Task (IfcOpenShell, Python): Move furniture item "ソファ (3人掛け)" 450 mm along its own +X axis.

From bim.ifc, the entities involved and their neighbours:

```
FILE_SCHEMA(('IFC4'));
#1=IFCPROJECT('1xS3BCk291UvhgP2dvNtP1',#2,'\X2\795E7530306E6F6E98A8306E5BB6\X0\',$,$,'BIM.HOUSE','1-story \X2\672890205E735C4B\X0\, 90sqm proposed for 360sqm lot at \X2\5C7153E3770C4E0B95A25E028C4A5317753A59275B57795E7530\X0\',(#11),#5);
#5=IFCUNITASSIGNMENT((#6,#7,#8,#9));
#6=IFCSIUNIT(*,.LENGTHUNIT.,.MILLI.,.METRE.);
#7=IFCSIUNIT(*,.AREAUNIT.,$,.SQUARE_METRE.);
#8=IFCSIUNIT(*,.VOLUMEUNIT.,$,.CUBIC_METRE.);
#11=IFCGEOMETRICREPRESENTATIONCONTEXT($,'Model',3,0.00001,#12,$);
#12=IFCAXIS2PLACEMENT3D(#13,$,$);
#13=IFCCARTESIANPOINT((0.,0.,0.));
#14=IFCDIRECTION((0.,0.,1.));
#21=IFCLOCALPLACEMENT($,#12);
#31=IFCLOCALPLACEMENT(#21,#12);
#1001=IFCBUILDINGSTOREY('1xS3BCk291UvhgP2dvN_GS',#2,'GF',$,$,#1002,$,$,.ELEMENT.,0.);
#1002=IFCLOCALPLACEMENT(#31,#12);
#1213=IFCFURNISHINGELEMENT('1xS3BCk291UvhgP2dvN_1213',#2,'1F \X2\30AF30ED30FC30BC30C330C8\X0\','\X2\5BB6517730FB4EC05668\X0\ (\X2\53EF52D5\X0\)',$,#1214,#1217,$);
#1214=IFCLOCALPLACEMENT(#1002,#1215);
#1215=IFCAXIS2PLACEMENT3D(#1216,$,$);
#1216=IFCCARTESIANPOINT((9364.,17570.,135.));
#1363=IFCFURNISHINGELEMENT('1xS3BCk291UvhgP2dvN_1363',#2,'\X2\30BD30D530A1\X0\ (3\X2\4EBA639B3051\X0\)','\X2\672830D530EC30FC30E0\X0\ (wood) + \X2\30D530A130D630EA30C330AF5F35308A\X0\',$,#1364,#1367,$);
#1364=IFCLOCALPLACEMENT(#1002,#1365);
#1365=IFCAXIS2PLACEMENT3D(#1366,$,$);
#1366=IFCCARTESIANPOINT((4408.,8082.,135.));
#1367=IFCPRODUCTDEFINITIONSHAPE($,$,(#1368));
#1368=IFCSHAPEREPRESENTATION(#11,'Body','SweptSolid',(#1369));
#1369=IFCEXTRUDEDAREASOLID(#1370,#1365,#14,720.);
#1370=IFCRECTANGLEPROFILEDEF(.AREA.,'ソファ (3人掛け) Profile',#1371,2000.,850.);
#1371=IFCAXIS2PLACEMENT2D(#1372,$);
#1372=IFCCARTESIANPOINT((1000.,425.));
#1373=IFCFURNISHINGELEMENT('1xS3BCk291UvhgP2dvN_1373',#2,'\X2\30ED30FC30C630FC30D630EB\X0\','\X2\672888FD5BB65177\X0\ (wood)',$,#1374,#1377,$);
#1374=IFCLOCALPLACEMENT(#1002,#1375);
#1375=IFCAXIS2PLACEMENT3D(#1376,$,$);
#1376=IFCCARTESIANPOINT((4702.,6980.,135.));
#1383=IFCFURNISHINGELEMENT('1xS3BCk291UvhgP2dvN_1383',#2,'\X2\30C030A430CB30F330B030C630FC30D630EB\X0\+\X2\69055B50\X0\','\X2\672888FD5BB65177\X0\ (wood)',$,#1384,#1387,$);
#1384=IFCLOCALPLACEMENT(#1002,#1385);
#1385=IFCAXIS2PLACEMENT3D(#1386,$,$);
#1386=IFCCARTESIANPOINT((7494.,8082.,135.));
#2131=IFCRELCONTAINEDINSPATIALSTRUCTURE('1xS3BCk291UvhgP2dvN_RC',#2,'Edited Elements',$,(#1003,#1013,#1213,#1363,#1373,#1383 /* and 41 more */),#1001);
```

```python
import ifcopenshell
import ifcopenshell.api.geometry
import ifcopenshell.util.placement

model = ifcopenshell.open("bim.ifc")

item = model.by_id(1363)
matrix = ifcopenshell.util.placement.get_local_placement(item.ObjectPlacement)
matrix[:3, 3] += matrix[:3, 0] * 450.0
ifcopenshell.api.geometry.edit_object_placement(model, product=item, matrix=matrix, is_si=False)

print(ifcopenshell.util.placement.get_local_placement(item.ObjectPlacement).round(3) + 0.0)

model.write("bim_edited.ifc")
```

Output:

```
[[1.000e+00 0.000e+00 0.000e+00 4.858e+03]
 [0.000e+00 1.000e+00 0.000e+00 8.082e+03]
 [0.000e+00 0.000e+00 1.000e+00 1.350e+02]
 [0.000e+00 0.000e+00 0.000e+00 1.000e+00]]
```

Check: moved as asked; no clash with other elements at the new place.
